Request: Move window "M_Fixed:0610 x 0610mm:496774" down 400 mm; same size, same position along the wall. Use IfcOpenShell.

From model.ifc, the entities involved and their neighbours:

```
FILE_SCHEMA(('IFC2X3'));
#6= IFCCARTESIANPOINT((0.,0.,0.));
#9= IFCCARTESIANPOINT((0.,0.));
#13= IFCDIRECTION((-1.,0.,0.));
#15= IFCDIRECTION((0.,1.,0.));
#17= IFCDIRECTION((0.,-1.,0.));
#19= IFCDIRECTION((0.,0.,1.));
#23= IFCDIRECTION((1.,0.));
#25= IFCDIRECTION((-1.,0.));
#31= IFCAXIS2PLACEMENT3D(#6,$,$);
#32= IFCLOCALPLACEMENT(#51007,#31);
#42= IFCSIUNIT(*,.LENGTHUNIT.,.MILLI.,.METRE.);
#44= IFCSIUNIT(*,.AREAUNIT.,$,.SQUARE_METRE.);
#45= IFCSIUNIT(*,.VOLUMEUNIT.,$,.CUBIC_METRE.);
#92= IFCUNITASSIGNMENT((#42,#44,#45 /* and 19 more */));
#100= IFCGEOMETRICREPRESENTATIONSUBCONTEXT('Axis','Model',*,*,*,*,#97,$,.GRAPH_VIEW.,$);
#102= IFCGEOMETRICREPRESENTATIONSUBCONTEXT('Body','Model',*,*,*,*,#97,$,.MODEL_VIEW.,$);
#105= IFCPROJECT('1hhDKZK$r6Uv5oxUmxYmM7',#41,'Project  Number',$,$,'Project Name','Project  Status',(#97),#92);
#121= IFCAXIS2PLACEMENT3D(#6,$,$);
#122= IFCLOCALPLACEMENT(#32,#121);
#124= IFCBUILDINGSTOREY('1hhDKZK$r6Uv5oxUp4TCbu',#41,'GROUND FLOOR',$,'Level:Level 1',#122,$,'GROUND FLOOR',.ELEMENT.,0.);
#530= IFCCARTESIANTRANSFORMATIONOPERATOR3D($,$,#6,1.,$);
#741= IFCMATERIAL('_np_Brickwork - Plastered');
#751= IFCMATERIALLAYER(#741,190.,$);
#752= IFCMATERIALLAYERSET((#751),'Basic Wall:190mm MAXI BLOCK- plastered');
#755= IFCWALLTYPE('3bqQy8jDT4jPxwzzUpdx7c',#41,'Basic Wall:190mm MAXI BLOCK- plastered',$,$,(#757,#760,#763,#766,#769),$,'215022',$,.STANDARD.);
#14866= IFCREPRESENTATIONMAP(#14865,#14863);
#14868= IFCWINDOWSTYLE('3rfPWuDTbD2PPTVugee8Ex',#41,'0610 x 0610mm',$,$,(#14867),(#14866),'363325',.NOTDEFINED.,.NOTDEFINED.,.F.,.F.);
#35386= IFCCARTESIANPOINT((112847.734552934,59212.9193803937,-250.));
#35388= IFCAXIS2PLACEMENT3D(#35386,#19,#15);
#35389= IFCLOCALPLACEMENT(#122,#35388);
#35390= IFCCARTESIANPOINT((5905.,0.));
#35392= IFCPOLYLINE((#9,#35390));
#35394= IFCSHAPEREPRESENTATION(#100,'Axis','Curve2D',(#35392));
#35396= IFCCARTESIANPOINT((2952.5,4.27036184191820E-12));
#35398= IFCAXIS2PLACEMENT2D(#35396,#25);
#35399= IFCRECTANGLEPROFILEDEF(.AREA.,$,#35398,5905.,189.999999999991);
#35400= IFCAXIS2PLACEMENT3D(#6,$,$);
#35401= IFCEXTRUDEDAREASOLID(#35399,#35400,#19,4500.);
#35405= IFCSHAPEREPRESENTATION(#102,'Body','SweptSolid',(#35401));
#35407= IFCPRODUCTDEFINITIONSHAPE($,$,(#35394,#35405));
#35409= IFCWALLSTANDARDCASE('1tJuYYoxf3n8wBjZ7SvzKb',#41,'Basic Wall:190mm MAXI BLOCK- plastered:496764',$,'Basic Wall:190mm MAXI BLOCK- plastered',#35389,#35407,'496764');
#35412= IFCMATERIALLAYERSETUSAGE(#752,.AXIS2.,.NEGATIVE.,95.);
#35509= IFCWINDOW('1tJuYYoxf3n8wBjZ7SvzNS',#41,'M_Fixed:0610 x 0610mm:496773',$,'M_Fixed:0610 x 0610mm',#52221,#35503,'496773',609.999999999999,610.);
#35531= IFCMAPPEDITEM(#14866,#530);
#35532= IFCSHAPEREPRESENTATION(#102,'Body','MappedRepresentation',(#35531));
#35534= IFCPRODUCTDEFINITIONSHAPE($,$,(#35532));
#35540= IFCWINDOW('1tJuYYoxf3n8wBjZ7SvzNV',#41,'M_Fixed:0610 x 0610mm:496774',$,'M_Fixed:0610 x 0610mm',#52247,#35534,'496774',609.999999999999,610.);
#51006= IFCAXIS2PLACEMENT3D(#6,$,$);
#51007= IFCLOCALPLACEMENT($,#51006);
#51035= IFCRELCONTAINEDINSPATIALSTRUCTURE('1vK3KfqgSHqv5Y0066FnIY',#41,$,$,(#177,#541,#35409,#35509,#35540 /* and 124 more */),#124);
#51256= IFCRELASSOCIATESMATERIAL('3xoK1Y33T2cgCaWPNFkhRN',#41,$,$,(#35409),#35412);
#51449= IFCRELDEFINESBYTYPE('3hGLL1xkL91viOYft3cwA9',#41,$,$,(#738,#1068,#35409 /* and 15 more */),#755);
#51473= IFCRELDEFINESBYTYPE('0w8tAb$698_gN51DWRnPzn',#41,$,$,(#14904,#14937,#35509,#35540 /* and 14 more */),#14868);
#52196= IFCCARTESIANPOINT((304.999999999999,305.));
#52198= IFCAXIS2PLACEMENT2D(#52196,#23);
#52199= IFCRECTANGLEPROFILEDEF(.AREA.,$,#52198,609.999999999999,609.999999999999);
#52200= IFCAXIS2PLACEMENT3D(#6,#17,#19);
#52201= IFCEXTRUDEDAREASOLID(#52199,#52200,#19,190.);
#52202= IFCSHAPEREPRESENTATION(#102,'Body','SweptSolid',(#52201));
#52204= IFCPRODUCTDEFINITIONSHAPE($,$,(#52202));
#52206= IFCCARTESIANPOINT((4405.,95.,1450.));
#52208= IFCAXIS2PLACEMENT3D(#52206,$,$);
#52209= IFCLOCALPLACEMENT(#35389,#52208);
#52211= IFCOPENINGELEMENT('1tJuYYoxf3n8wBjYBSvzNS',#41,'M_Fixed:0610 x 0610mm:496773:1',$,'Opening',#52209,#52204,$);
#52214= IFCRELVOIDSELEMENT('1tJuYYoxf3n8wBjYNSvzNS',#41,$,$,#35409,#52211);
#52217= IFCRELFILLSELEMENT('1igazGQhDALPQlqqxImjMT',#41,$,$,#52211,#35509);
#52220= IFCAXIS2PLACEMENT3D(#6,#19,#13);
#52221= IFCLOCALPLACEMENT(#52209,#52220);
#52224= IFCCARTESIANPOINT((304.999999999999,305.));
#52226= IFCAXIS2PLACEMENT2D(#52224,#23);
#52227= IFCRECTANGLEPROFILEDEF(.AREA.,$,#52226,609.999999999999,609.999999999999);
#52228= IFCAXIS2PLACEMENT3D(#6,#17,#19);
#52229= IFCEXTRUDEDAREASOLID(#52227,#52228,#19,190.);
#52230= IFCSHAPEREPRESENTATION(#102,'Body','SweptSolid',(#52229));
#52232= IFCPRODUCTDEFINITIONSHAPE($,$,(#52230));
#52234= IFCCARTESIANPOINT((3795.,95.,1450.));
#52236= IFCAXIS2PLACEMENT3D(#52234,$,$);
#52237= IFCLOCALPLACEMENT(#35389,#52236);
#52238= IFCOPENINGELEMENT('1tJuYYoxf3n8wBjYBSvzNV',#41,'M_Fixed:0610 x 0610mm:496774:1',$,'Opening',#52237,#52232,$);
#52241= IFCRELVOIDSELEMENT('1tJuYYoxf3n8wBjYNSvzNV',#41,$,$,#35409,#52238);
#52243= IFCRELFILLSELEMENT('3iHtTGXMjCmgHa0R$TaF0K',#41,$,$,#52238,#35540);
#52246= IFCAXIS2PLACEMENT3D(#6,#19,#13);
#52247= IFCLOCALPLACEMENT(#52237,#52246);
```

```python
import numpy as np
import ifcopenshell
import ifcopenshell.api.geometry
import ifcopenshell.util.placement
import ifcopenshell.util.unit

model = ifcopenshell.open("model.ifc")
unit_scale = ifcopenshell.util.unit.calculate_unit_scale(model)

window = model.by_guid("1tJuYYoxf3n8wBjZ7SvzNV")
opening = window.FillsVoids[0].RelatingOpeningElement
dz = -400.0

shift = np.array([0.0, 0.0, dz])
# The window is placed relative to its opening, so it follows when the opening moves.
matrix = ifcopenshell.util.placement.get_local_placement(opening.ObjectPlacement)
matrix[:3, 3] += shift
ifcopenshell.api.geometry.edit_object_placement(
    model, product=opening, matrix=matrix, is_si=False, should_transform_children=True
)

print(f"moved by {dz * unit_scale:+.3f} m")

model.write("model_rev.ifc")
```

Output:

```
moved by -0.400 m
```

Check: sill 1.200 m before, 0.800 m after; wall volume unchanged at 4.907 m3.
